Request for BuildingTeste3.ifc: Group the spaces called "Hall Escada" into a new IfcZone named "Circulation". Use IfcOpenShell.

First a look at what the model holds.

```python
import ifcopenshell

model = ifcopenshell.open("BuildingTeste3.ifc")
print(model.schema)
seen = {}
for space in model.by_type("IfcSpace"):
    seen[space.LongName] = seen.get(space.LongName, 0) + 1
for name, count in sorted(seen.items(), key=str):
    print(count, "x", name)
print("zones:", [z.Name for z in model.by_type("IfcZone")][:20])
```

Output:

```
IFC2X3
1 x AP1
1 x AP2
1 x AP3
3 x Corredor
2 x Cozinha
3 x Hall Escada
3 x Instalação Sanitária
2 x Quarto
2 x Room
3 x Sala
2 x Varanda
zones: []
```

```python
import ifcopenshell
import ifcopenshell.api.group
import ifcopenshell.api.root

model = ifcopenshell.open("BuildingTeste3.ifc")

names = {"Hall Escada"}
spaces = [s for s in model.by_type("IfcSpace") if s.LongName in names]

zone = ifcopenshell.api.root.create_entity(model, ifc_class="IfcZone", name="Circulation")
ifcopenshell.api.group.assign_group(model, products=spaces, group=zone)
print(len(spaces), "spaces in", zone.Name)

model.write("BuildingTeste3_v2.ifc")
```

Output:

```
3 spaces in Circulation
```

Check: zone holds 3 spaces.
